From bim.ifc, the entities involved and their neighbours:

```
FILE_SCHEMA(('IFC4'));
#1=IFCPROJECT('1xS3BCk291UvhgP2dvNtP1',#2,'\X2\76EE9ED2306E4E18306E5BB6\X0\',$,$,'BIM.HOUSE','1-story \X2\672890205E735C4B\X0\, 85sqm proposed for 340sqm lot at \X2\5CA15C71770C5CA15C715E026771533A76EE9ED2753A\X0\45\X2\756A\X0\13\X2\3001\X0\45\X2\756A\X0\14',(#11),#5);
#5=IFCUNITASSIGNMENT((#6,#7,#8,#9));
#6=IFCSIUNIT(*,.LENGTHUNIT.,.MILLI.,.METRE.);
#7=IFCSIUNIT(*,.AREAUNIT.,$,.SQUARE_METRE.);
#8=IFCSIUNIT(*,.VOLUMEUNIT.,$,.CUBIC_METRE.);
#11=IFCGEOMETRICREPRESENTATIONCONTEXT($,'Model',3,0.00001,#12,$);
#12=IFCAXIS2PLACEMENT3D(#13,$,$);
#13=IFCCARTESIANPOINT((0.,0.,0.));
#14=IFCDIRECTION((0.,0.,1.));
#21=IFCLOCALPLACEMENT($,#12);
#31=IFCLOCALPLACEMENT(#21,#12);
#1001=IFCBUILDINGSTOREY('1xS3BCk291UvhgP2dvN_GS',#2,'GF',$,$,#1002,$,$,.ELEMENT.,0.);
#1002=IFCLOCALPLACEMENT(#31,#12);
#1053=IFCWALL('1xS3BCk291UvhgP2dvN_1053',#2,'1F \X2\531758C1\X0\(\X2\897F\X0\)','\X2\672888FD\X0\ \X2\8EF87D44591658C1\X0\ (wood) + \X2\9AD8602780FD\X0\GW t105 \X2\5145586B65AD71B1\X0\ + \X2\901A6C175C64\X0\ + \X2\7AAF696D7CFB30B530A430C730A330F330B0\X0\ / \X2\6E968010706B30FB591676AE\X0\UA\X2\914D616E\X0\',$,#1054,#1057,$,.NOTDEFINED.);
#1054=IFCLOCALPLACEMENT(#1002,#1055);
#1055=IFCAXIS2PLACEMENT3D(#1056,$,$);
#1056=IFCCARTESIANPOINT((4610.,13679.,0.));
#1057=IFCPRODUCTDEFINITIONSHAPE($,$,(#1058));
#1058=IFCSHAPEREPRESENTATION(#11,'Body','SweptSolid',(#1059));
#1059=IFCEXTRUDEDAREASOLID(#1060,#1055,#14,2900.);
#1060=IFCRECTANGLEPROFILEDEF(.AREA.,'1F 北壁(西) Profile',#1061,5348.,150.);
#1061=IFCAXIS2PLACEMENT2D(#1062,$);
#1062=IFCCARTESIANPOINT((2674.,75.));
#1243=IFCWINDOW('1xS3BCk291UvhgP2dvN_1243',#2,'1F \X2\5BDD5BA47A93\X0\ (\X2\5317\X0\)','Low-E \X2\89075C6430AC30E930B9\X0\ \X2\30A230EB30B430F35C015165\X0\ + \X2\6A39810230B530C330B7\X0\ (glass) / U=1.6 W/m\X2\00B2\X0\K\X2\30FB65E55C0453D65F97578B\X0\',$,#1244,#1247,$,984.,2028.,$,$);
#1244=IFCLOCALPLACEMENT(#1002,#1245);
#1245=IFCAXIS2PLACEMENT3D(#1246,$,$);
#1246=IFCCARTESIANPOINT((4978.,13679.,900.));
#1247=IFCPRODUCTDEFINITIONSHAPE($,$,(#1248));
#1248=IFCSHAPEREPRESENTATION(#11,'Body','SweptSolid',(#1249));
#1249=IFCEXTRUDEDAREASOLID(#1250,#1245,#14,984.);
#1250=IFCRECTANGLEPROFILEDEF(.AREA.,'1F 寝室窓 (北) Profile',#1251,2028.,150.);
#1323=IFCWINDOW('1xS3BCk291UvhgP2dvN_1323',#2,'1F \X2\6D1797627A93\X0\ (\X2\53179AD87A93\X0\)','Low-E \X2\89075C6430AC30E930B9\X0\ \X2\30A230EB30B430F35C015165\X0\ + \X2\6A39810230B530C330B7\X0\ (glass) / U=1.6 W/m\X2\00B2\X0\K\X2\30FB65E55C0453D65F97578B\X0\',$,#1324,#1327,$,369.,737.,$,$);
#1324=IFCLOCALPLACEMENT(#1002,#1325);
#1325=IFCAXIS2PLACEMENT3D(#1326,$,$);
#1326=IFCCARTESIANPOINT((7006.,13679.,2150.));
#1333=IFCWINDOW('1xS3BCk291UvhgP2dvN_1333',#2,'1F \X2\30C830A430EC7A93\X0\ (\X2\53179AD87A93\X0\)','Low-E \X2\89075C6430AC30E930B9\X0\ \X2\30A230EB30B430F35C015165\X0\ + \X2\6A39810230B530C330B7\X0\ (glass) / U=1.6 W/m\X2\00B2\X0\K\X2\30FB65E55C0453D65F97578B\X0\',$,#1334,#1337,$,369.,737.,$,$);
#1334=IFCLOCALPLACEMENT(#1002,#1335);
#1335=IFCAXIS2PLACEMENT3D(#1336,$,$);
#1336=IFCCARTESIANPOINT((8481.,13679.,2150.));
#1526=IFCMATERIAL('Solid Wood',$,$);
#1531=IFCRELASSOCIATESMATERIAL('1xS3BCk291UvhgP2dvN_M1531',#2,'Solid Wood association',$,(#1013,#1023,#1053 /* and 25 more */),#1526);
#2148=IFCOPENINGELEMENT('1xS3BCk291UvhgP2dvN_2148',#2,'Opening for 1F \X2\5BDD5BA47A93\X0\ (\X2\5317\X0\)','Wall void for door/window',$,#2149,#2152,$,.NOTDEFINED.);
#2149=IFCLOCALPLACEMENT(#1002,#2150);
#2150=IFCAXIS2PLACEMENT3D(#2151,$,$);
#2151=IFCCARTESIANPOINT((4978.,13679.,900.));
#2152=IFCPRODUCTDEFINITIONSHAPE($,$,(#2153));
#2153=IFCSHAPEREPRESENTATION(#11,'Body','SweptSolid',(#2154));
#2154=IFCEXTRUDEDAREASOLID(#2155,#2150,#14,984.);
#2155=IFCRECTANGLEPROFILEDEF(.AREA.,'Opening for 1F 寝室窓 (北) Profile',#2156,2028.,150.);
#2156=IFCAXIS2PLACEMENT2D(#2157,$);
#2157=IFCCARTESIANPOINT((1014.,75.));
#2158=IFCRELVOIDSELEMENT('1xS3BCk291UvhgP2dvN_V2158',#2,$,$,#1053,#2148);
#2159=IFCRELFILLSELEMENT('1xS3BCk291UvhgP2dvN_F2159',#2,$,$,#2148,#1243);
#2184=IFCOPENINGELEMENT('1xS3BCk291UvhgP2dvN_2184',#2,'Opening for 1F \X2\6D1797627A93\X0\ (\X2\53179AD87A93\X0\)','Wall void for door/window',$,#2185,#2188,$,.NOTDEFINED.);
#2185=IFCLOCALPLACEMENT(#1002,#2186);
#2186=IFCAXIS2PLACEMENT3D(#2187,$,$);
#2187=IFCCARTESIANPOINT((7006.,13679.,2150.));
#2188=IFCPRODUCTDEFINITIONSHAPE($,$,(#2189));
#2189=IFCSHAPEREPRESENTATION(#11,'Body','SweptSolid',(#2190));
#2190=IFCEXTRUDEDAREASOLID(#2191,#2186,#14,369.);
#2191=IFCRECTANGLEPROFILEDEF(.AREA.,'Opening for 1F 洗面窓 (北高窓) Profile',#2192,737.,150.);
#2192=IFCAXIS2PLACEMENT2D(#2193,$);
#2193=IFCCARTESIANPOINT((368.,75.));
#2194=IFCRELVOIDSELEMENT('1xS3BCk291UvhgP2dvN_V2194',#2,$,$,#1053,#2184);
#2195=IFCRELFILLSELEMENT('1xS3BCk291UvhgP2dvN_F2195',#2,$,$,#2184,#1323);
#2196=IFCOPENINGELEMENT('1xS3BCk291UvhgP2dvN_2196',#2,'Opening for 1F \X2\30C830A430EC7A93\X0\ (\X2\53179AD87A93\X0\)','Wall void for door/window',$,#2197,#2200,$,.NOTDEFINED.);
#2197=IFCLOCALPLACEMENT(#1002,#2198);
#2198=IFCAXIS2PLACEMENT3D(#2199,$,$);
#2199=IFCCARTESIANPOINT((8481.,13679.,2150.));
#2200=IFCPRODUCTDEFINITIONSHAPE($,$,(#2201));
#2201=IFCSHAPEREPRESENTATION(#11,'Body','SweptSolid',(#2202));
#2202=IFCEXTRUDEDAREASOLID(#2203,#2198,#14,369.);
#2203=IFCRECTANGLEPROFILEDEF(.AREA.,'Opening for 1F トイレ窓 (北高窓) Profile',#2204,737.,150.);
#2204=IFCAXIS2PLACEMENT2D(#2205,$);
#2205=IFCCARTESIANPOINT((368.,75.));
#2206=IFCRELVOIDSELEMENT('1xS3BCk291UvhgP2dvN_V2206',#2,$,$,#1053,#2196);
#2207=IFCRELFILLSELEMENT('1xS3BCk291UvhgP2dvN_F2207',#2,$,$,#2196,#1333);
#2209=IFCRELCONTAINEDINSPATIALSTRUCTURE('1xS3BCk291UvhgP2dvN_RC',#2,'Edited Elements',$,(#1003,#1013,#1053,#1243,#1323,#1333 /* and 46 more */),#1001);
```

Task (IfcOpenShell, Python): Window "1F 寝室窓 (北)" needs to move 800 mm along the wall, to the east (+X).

```python
import ifcopenshell
import ifcopenshell.api.geometry
import ifcopenshell.util.placement

model = ifcopenshell.open("bim.ifc")

window = model.by_guid("1xS3BCk291UvhgP2dvN_1243")
opening = window.FillsVoids[0].RelatingOpeningElement
wall = opening.VoidsElements[0].RelatingBuildingElement

wall_matrix = ifcopenshell.util.placement.get_local_placement(wall.ObjectPlacement)
shift = wall_matrix[:3, 0] * 800.0
before = ifcopenshell.util.placement.get_local_placement(window.ObjectPlacement)[:3, 3].copy()

# The window is not placed relative to its opening, so move both.
for product in (opening, window):
    matrix = ifcopenshell.util.placement.get_local_placement(product.ObjectPlacement)
    matrix[:3, 3] += shift
    ifcopenshell.api.geometry.edit_object_placement(model, product=product, matrix=matrix, is_si=False)

after = ifcopenshell.util.placement.get_local_placement(window.ObjectPlacement)[:3, 3]
print("window moved by", (after - before).round(3) + 0.0)

model.write("bim_v2.ifc")
```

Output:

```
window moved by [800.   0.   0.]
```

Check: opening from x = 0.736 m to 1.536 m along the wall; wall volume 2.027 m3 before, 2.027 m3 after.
